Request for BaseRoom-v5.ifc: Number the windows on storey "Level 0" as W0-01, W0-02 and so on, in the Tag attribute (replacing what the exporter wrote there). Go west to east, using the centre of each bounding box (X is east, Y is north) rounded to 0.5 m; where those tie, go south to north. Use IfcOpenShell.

First a look at what the model holds.

```python
import ifcopenshell
import ifcopenshell.util.element
import ifcopenshell.util.placement

model = ifcopenshell.open("BaseRoom-v5.ifc")
print(model.schema)
storey = next(s for s in model.by_type("IfcBuildingStorey") if s.Name == "Level 0")
windows = [e for e in ifcopenshell.util.element.get_decomposition(storey) if e.is_a("IfcWindow")]
for e in sorted(windows, key=lambda e: e.id()):
    origin = ifcopenshell.util.placement.get_local_placement(e.ObjectPlacement)[:3, 3]
    print(e.id(), e.Tag, e.Name, origin.round(2) + 0.0, sep=" | ")
```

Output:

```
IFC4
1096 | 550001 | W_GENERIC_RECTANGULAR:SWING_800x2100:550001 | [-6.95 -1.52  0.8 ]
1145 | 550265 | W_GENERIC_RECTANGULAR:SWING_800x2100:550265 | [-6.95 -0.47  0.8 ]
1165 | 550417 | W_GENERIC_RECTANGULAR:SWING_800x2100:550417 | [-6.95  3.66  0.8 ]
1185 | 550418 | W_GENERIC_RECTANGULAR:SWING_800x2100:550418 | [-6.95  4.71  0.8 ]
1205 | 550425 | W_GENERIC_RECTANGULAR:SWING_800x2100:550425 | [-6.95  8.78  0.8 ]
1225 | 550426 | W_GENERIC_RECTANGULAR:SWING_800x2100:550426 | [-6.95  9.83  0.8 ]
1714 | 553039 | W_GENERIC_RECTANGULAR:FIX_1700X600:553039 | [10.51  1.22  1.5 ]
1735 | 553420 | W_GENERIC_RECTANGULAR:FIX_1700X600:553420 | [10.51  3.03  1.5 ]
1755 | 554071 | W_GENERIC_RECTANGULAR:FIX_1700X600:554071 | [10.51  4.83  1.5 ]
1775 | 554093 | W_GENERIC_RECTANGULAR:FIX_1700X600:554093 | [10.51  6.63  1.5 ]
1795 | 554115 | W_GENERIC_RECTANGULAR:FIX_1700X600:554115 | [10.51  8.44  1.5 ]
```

```python
import ifcopenshell
import ifcopenshell.geom
import ifcopenshell.util.element
import ifcopenshell.util.shape

model = ifcopenshell.open("BaseRoom-v5.ifc")
settings = ifcopenshell.geom.settings()
settings.set("use-world-coords", True)


def centre(element):
    shape = ifcopenshell.geom.create_shape(settings, element)
    return ifcopenshell.util.shape.get_bbox_centroid(shape.geometry)


storey = next(s for s in model.by_type("IfcBuildingStorey") if s.Name == "Level 0")
windows = [e for e in ifcopenshell.util.element.get_decomposition(storey) if e.is_a("IfcWindow")]

# Insertion points can sit at a corner or the storey origin, so sort by the geometry (in metres).
centres = {e: centre(e) for e in windows}
windows.sort(key=lambda e: (round(centres[e][0] / 0.5), centres[e][1]))

for i, e in enumerate(windows, start=1):
    number = f"W0-{i:02d}"
    e.Tag = number
    print(e.id(), number)

model.write("BaseRoom-v5-out.ifc")
```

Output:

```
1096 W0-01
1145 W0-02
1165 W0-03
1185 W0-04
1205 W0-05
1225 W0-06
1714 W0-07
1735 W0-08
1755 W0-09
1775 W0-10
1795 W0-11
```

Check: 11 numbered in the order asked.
